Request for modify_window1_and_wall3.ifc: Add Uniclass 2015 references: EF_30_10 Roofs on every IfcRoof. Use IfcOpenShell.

First a look at what the model holds.

```python
import ifcopenshell

model = ifcopenshell.open("modify_window1_and_wall3.ifc")
print(model.schema)
print("classifications:", [c.Name for c in model.by_type("IfcClassification")])
for ifc_class in ("IfcDoor", "IfcRoof", "IfcStair", "IfcWall", "IfcWindow"):
    print(ifc_class, len(model.by_type(ifc_class)))
```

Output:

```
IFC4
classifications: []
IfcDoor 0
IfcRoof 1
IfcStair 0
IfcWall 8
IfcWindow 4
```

```python
import ifcopenshell
import ifcopenshell.api.classification

model = ifcopenshell.open("modify_window1_and_wall3.ifc")

system = ifcopenshell.api.classification.add_classification(model, classification="Uniclass 2015")

codes = {
    "IfcRoof": ("EF_30_10", "Roofs"),
}
for ifc_class, (code, name) in codes.items():
    products = model.by_type(ifc_class)
    ifcopenshell.api.classification.add_reference(
        model, products=products, classification=system, identification=code, name=name
    )
    print(code, len(products))

model.write("modify_window1_and_wall3_v2.ifc")
```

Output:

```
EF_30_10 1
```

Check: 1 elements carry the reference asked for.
